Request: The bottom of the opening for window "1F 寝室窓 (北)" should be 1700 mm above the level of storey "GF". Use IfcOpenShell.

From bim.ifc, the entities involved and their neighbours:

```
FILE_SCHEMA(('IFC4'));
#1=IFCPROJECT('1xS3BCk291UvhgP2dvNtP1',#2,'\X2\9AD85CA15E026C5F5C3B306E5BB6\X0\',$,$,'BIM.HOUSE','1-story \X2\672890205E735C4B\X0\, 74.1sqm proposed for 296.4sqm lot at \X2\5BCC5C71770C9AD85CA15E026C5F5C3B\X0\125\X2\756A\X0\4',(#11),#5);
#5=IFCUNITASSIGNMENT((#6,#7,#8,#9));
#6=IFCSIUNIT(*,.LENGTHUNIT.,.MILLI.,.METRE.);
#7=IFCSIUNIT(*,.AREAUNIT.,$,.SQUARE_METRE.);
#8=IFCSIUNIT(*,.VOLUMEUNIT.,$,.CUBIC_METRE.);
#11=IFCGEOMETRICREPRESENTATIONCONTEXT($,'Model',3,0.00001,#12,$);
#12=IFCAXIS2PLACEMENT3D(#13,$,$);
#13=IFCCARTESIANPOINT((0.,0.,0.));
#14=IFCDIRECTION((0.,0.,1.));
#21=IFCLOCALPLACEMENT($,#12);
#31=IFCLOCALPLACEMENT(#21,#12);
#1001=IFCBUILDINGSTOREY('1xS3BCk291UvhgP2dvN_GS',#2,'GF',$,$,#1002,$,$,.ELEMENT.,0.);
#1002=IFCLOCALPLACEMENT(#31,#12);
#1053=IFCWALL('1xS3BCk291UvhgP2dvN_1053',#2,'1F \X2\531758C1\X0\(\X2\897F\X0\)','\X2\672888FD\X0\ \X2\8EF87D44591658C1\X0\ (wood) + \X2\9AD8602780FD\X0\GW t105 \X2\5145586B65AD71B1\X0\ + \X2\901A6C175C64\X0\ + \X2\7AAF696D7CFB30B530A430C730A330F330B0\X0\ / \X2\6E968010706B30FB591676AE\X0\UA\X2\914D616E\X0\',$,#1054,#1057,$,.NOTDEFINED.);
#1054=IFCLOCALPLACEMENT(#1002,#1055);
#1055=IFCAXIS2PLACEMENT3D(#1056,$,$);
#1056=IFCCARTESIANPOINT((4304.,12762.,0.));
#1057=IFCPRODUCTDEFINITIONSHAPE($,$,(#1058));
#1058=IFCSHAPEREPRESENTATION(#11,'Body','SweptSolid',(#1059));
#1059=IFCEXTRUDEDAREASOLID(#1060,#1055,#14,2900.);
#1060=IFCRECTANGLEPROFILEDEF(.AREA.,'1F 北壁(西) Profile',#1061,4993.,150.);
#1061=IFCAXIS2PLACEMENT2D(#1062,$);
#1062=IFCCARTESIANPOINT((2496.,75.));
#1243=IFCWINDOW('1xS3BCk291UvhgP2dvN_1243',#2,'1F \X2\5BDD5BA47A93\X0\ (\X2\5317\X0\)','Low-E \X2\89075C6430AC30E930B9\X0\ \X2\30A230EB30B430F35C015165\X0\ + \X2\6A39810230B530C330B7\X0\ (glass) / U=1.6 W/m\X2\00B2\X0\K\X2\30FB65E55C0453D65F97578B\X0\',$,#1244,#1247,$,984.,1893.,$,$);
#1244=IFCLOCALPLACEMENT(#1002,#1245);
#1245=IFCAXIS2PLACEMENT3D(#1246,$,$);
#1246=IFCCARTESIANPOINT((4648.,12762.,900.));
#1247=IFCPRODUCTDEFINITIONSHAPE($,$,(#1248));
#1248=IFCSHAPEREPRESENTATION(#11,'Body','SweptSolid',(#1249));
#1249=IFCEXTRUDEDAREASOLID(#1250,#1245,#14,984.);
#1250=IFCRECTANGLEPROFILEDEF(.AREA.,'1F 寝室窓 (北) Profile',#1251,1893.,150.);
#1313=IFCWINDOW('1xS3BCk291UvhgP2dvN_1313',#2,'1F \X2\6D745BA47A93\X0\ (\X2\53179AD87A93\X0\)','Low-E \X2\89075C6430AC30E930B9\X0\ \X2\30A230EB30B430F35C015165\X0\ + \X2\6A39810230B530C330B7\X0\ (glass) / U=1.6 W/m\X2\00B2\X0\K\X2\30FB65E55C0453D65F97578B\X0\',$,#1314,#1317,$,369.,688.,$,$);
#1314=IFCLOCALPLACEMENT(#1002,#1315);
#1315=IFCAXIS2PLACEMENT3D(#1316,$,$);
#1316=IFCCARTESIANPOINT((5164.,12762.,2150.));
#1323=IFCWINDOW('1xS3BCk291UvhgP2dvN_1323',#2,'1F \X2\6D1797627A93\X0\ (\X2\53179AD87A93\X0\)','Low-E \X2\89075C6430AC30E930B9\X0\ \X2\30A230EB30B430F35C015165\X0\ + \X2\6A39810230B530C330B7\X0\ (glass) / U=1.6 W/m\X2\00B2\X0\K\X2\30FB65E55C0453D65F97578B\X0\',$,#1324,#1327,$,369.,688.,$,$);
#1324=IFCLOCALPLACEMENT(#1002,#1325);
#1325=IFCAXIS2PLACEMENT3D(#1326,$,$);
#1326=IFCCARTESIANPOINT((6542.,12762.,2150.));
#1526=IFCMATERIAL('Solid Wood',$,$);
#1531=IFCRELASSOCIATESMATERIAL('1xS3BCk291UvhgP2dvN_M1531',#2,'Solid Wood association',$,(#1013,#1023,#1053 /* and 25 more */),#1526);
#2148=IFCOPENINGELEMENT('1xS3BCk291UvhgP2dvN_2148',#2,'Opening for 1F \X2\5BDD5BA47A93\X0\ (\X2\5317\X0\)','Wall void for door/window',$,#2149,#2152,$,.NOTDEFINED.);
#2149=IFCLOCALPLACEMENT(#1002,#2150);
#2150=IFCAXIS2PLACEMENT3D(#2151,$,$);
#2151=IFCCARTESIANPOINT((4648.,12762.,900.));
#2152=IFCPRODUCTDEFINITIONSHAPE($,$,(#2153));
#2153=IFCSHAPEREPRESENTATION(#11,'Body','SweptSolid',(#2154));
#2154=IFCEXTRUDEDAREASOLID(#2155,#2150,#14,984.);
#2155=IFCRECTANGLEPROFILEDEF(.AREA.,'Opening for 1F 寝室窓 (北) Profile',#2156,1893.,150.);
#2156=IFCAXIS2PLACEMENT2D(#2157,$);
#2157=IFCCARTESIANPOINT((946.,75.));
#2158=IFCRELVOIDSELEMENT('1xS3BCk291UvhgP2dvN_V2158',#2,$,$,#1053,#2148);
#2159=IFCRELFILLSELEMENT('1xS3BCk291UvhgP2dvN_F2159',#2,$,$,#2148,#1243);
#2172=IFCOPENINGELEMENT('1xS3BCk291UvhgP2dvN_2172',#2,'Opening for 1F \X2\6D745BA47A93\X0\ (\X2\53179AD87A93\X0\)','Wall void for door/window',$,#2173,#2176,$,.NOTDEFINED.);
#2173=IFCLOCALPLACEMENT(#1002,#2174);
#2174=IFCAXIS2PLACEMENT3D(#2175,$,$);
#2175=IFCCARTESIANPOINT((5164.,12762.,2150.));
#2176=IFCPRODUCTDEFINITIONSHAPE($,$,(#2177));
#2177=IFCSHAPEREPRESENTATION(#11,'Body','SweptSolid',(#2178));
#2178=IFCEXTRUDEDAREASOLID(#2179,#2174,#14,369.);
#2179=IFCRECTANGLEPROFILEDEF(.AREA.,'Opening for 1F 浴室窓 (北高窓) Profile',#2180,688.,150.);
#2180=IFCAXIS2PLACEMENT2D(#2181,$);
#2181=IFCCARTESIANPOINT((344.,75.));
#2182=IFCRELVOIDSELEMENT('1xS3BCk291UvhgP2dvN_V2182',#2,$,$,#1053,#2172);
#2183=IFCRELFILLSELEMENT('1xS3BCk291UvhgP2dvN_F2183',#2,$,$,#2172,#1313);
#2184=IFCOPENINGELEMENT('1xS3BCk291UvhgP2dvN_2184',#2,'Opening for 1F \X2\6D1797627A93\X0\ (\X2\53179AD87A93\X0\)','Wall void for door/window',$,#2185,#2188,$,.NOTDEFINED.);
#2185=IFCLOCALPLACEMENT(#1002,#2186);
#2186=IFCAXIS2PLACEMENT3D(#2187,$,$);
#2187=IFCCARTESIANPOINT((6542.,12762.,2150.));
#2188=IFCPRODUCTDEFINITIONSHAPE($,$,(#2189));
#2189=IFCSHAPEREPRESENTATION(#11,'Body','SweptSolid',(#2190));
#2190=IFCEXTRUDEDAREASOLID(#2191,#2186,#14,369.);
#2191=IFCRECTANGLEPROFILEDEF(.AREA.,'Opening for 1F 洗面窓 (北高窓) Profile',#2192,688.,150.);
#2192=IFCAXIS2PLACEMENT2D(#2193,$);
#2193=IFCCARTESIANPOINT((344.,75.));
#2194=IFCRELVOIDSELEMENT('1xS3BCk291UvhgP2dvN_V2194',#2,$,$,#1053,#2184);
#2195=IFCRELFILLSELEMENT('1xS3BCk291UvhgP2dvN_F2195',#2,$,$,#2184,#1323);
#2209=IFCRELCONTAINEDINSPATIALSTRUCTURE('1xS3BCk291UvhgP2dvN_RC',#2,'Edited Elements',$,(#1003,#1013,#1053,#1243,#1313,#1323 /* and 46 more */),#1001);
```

```python
import numpy as np
import ifcopenshell
import ifcopenshell.api.geometry
import ifcopenshell.geom
import ifcopenshell.util.element
import ifcopenshell.util.placement
import ifcopenshell.util.shape
import ifcopenshell.util.unit

model = ifcopenshell.open("bim.ifc")
unit_scale = ifcopenshell.util.unit.calculate_unit_scale(model)

window = model.by_id(1243)
opening = window.FillsVoids[0].RelatingOpeningElement
storey = ifcopenshell.util.element.get_container(window, ifc_class="IfcBuildingStorey")
level = ifcopenshell.util.placement.get_local_placement(storey.ObjectPlacement)[2, 3]

# The opening's origin need not be at the sill, so measure its lowest point.
shape = ifcopenshell.geom.create_shape(ifcopenshell.geom.settings(), opening)
bottom = ifcopenshell.util.shape.get_shape_bottom_elevation(shape, shape.geometry) / unit_scale
dz = level + 1.7 / unit_scale - bottom

shift = np.array([0.0, 0.0, dz])
# The window is not placed relative to its opening, so move both.
for product in (opening, window):
    matrix = ifcopenshell.util.placement.get_local_placement(product.ObjectPlacement)
    matrix[:3, 3] += shift
    ifcopenshell.api.geometry.edit_object_placement(model, product=product, matrix=matrix, is_si=False)

print(f"moved by {dz * unit_scale:+.3f} m")

model.write("bim-out.ifc")
```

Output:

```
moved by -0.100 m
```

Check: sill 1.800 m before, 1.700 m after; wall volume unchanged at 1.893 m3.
